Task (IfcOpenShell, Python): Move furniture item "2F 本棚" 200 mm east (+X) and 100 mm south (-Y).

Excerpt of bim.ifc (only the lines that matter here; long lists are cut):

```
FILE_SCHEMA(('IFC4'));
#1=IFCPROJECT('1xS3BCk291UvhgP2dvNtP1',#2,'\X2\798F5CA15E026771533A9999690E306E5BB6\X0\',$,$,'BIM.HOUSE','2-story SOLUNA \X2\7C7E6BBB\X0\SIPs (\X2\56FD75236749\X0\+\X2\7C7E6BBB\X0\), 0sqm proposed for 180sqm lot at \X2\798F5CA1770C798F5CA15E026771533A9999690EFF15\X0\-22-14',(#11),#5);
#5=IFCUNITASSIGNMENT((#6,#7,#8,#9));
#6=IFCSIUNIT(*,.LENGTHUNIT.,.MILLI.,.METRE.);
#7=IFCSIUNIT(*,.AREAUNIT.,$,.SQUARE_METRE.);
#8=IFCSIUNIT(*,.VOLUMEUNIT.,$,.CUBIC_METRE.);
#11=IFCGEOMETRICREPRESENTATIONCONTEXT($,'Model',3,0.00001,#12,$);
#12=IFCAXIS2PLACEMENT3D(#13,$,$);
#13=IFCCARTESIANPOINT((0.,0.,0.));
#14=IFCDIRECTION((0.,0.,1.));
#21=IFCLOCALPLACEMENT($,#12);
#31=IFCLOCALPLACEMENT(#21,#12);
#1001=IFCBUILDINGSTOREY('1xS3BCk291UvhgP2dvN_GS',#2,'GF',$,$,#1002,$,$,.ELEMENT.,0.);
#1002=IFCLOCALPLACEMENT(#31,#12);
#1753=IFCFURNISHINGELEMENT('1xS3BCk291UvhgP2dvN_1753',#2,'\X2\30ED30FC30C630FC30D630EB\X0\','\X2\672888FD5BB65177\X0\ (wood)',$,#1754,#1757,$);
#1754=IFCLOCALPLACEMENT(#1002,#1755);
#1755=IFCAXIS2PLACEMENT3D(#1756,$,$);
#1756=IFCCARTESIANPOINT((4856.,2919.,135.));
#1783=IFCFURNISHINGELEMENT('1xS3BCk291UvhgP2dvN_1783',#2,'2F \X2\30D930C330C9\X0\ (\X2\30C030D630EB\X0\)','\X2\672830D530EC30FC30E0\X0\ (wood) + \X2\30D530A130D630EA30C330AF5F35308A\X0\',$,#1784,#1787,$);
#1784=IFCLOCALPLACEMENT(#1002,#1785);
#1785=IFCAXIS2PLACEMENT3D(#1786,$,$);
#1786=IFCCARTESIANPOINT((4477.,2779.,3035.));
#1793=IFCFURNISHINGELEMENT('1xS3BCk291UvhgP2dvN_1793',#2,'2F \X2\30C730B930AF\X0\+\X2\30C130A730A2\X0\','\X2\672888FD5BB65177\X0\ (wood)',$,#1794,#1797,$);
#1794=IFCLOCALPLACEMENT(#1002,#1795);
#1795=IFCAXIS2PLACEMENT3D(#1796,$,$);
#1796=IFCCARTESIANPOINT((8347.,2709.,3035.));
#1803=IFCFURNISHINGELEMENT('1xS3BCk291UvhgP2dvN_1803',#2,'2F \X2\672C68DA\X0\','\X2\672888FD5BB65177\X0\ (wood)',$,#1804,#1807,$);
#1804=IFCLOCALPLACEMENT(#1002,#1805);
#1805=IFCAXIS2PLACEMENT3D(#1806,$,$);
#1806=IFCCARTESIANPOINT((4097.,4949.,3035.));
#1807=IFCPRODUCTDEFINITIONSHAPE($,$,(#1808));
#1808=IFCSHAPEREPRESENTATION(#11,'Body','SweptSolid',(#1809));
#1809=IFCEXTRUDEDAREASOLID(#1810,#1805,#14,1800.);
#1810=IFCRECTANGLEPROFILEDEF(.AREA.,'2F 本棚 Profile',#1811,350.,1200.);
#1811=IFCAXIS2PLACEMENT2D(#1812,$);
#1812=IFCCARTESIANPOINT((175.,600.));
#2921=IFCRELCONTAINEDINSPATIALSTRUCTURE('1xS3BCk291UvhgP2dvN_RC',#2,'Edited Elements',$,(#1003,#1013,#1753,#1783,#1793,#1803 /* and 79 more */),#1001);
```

```python
import ifcopenshell
import ifcopenshell.api.geometry
import ifcopenshell.util.placement
import ifcopenshell.util.unit

model = ifcopenshell.open("bim.ifc")
unit_scale = ifcopenshell.util.unit.calculate_unit_scale(model)

item = model.by_id(1803)
matrix = ifcopenshell.util.placement.get_local_placement(item.ObjectPlacement)
matrix[0, 3] += 0.2 / unit_scale
matrix[1, 3] -= 0.1 / unit_scale
ifcopenshell.api.geometry.edit_object_placement(model, product=item, matrix=matrix, is_si=False)

print(ifcopenshell.util.placement.get_local_placement(item.ObjectPlacement).round(3) + 0.0)

model.write("bim_rev.ifc")
```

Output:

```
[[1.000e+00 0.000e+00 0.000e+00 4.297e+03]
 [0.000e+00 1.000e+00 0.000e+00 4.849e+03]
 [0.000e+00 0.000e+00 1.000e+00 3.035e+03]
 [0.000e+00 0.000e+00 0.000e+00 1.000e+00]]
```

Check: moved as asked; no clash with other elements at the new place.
